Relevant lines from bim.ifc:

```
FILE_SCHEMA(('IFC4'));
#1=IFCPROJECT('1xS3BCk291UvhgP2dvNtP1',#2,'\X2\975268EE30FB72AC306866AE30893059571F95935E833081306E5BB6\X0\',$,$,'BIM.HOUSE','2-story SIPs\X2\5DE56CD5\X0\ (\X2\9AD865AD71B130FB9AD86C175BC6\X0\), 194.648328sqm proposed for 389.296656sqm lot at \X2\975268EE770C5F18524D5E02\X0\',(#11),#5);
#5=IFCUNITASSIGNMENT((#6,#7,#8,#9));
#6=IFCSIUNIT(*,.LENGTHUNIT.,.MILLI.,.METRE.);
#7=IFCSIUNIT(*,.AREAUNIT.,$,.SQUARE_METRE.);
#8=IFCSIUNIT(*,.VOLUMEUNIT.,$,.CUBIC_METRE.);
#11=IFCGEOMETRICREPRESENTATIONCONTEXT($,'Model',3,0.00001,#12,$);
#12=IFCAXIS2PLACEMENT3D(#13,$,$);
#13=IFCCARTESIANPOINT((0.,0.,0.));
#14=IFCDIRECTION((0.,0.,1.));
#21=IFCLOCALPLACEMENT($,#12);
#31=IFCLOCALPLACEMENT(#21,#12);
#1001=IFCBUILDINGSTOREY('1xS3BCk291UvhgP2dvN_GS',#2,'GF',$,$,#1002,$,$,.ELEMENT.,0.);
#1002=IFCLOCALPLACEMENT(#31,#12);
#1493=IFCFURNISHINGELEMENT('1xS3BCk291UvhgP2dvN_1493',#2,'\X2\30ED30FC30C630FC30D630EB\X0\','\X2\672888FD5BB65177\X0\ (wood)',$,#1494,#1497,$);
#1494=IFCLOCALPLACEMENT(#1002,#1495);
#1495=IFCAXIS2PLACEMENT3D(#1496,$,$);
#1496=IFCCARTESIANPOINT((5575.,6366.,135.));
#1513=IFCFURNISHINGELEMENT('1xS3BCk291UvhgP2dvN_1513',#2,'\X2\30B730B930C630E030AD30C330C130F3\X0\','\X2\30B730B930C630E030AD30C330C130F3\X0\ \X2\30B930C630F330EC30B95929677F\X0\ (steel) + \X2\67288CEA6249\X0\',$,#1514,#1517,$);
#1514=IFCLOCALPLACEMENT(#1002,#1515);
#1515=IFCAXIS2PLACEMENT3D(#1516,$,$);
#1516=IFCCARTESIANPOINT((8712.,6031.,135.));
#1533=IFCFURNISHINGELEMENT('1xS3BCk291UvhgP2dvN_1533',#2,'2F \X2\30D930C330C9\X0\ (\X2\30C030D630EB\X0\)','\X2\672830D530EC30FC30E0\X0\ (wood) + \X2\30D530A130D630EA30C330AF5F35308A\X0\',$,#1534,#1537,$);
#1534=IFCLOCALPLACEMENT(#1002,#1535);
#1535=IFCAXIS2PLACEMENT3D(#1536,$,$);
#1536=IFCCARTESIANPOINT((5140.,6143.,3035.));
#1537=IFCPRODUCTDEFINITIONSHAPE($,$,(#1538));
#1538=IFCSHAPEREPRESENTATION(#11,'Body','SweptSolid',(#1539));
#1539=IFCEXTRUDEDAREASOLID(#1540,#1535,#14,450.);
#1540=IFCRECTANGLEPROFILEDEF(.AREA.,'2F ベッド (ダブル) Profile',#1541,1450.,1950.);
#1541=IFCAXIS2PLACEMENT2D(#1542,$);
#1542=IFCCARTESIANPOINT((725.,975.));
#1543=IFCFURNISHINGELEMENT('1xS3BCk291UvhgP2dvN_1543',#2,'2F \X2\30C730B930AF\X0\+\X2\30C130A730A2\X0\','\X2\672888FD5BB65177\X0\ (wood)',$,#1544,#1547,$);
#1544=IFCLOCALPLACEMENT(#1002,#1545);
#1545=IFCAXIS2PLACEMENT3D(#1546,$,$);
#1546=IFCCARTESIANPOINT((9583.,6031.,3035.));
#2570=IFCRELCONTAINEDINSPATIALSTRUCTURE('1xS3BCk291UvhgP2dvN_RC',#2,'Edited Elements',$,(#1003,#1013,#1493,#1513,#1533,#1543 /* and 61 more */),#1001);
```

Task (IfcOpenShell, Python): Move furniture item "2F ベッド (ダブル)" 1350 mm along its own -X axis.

```python
import ifcopenshell
import ifcopenshell.api.geometry
import ifcopenshell.util.placement
import ifcopenshell.util.unit

model = ifcopenshell.open("bim.ifc")
unit_scale = ifcopenshell.util.unit.calculate_unit_scale(model)

item = model.by_guid("1xS3BCk291UvhgP2dvN_1533")
matrix = ifcopenshell.util.placement.get_local_placement(item.ObjectPlacement)
matrix[:3, 3] -= matrix[:3, 0] * 1.35 / unit_scale
ifcopenshell.api.geometry.edit_object_placement(model, product=item, matrix=matrix, is_si=False)

print(ifcopenshell.util.placement.get_local_placement(item.ObjectPlacement).round(3) + 0.0)

model.write("bim_rev.ifc")
```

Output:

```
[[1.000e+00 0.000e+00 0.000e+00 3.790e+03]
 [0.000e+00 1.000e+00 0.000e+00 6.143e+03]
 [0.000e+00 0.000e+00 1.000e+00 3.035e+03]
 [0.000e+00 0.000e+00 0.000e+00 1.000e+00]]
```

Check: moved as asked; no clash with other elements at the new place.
